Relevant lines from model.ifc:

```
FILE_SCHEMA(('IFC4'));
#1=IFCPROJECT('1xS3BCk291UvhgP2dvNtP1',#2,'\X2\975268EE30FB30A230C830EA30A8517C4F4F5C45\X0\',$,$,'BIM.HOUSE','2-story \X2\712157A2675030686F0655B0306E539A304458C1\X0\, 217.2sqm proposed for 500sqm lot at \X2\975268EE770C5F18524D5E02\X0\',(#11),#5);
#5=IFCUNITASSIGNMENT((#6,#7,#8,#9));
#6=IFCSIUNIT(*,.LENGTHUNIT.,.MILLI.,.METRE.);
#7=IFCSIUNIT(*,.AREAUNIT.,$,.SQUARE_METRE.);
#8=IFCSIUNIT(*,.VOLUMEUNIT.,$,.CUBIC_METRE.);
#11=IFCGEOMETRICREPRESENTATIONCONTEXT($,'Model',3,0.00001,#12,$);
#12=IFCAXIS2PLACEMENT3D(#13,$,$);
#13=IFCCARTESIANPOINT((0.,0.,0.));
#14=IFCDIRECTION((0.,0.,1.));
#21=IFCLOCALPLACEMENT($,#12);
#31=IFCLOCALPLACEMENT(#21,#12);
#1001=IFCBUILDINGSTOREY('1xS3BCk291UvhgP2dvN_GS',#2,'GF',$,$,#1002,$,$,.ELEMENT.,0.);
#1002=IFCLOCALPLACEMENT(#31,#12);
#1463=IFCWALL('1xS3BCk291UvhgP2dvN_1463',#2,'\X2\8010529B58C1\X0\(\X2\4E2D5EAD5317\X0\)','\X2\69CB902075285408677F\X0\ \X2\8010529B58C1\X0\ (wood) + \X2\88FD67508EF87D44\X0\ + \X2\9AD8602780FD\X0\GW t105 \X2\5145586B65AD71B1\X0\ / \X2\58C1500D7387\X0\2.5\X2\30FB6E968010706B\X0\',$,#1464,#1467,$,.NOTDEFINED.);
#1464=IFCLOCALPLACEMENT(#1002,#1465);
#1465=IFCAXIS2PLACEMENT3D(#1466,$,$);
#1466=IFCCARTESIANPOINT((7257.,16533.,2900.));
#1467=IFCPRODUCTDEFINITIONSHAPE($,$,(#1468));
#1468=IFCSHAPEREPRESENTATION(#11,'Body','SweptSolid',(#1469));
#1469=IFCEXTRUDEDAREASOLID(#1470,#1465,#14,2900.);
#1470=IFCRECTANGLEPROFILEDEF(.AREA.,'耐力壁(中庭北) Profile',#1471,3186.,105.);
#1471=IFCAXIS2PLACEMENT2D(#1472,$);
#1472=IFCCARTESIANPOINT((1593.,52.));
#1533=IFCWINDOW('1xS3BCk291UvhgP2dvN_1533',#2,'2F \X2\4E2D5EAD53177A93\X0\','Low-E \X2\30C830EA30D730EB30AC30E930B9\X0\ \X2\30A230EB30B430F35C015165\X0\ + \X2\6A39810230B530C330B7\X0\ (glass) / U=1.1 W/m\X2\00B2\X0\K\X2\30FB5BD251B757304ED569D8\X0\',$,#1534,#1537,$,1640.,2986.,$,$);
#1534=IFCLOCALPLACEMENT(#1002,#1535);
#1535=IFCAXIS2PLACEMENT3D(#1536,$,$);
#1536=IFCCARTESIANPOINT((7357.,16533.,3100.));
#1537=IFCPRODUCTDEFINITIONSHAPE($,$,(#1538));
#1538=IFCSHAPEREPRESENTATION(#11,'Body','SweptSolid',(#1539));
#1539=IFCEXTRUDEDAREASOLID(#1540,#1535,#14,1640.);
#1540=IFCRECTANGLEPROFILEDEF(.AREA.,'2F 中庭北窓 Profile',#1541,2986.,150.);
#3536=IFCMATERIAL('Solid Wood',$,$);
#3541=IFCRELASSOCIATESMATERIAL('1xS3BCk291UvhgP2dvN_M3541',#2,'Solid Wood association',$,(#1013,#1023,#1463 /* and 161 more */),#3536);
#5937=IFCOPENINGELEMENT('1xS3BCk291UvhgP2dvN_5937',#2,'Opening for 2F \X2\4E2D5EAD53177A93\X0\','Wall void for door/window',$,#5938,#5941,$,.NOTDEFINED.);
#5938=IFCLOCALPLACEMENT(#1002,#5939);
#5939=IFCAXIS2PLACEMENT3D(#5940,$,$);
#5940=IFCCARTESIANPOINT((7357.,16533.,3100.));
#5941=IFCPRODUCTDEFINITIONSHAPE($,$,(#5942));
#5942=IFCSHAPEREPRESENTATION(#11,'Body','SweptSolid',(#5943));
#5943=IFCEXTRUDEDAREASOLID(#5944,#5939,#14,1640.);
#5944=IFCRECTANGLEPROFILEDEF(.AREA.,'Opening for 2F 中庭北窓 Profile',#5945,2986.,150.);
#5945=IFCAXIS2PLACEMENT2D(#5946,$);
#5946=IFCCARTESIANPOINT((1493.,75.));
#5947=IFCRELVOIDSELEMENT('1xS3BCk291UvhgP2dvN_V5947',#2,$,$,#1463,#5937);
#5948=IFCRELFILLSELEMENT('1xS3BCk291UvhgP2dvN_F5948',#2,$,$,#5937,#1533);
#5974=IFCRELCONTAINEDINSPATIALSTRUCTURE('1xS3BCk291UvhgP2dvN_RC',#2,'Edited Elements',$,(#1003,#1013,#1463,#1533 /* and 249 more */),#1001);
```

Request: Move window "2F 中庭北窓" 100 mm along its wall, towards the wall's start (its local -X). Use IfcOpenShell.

```python
import ifcopenshell
import ifcopenshell.api.geometry
import ifcopenshell.util.placement
import ifcopenshell.util.unit

model = ifcopenshell.open("model.ifc")
unit_scale = ifcopenshell.util.unit.calculate_unit_scale(model)

window = model.by_guid("1xS3BCk291UvhgP2dvN_1533")
opening = window.FillsVoids[0].RelatingOpeningElement
wall = opening.VoidsElements[0].RelatingBuildingElement

wall_matrix = ifcopenshell.util.placement.get_local_placement(wall.ObjectPlacement)
shift = wall_matrix[:3, 0] * -0.1 / unit_scale
before = ifcopenshell.util.placement.get_local_placement(window.ObjectPlacement)[:3, 3].copy()

# The window is not placed relative to its opening, so move both.
for product in (opening, window):
    matrix = ifcopenshell.util.placement.get_local_placement(product.ObjectPlacement)
    matrix[:3, 3] += shift
    ifcopenshell.api.geometry.edit_object_placement(model, product=product, matrix=matrix, is_si=False)

after = ifcopenshell.util.placement.get_local_placement(window.ObjectPlacement)[:3, 3]
print("window moved by", (after - before).round(3) + 0.0)

model.write("model_v2.ifc")
```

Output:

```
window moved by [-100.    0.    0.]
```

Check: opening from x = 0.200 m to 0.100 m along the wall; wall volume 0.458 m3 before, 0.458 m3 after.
